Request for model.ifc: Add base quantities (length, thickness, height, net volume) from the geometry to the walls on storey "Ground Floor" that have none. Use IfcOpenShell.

First a look at what the model holds.

```python
import ifcopenshell
import ifcopenshell.util.element
import ifcopenshell.util.unit

model = ifcopenshell.open("model.ifc")
print(model.schema)
for unit_type in ("LENGTHUNIT", "AREAUNIT", "VOLUMEUNIT"):
    print(unit_type, ifcopenshell.util.unit.calculate_unit_scale(model, unit_type))
storey = next(s for s in model.by_type("IfcBuildingStorey") if s.Name == "Ground Floor")
walls = [e for e in ifcopenshell.util.element.get_decomposition(storey) if e.is_a("IfcWall")]
for e in sorted(walls, key=lambda e: e.id()):
    print(e.id(), e.is_a(), e.Name, list(ifcopenshell.util.element.get_psets(e, qtos_only=True)), sep=" | ")
```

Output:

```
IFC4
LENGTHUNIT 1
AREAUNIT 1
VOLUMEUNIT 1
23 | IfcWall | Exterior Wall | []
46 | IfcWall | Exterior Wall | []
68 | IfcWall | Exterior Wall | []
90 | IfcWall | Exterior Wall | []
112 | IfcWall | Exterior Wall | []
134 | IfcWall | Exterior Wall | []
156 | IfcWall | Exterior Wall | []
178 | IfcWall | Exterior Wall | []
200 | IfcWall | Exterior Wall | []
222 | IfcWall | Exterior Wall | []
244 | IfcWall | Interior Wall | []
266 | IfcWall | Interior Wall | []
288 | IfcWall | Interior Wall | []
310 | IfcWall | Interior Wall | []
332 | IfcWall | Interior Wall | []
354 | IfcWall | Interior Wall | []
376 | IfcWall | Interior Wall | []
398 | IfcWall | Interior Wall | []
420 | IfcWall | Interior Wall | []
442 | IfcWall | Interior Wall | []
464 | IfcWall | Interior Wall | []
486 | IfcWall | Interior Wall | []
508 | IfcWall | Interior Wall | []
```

```python
import ifcopenshell
import ifcopenshell.api.pset
import ifcopenshell.geom
import ifcopenshell.util.element
import ifcopenshell.util.shape
import ifcopenshell.util.unit

model = ifcopenshell.open("model.ifc")
unit_scale = ifcopenshell.util.unit.calculate_unit_scale(model)
volume_scale = ifcopenshell.util.unit.calculate_unit_scale(model, "VOLUMEUNIT")
settings = ifcopenshell.geom.settings()

storey = next(s for s in model.by_type("IfcBuildingStorey") if s.Name == "Ground Floor")
walls = [e for e in ifcopenshell.util.element.get_decomposition(storey) if e.is_a("IfcWall")]

for e in sorted(walls, key=lambda e: e.id()):
    if ifcopenshell.util.element.get_psets(e, qtos_only=True, should_inherit=False):
        continue
    # Geometry comes back in metres, in the element's own axes.
    shape = ifcopenshell.geom.create_shape(settings, e)
    values = {
        "Length": ifcopenshell.util.shape.get_x(shape.geometry) / unit_scale,
        "Width": ifcopenshell.util.shape.get_y(shape.geometry) / unit_scale,
        "Height": ifcopenshell.util.shape.get_z(shape.geometry) / unit_scale,
        "NetVolume": ifcopenshell.util.shape.get_volume(shape.geometry) / volume_scale,
    }
    qto = ifcopenshell.api.pset.add_qto(model, product=e, name="Qto_WallBaseQuantities")
    ifcopenshell.api.pset.edit_qto(model, qto=qto, properties=values)
    print(e.id(), {k: round(v, 3) for k, v in values.items()})

model.write("model_updated.ifc")
```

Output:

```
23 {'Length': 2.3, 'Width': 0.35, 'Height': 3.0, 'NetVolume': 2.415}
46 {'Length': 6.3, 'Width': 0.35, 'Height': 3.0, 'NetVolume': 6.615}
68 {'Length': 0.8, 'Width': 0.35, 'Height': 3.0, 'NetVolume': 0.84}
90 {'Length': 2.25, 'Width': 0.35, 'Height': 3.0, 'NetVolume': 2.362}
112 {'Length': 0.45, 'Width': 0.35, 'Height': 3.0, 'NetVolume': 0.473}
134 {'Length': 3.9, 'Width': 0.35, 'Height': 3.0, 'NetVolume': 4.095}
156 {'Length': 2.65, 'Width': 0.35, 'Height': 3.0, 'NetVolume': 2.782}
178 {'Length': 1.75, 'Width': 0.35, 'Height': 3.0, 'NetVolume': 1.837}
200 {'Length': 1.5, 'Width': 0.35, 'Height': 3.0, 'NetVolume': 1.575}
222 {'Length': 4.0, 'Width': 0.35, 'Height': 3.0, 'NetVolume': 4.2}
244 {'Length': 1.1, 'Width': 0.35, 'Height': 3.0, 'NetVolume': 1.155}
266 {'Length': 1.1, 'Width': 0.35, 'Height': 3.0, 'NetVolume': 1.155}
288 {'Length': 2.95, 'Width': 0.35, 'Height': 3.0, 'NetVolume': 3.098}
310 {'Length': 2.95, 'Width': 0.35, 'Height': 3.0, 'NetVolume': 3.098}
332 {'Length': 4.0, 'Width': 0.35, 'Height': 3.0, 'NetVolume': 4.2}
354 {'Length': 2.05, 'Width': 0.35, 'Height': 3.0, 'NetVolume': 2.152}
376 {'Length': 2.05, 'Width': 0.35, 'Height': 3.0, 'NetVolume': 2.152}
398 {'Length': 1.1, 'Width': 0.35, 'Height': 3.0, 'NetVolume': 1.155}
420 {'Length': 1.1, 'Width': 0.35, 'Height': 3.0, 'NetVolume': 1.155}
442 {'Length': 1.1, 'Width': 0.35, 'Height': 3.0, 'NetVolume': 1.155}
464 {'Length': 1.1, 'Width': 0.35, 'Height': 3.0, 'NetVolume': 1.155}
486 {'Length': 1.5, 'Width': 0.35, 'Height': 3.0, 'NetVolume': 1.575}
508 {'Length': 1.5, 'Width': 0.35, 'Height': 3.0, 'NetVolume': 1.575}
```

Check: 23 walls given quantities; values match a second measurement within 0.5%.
